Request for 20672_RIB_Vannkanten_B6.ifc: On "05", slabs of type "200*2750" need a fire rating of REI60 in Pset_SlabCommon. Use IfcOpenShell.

First a look at what the model holds.

```python
import ifcopenshell
import ifcopenshell.util.element

model = ifcopenshell.open("20672_RIB_Vannkanten_B6.ifc")
print(model.schema)
storey = next(s for s in model.by_type("IfcBuildingStorey") if s.Name == "05")
slabs = [e for e in ifcopenshell.util.element.get_decomposition(storey) if e.is_a("IfcSlab")]
seen = {}
for e in slabs:
    element_type = ifcopenshell.util.element.get_type(e)
    key = (element_type.Name if element_type != e and element_type else None, ifcopenshell.util.element.get_pset(e, "Pset_SlabCommon", "FireRating"))
    seen[key] = seen.get(key, 0) + 1
for (name, value), count in sorted(seen.items(), key=str):
    print(count, "x", name, "|", value)
```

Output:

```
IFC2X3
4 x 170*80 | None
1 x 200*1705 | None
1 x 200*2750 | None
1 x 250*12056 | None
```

```python
import ifcopenshell
import ifcopenshell.api.pset
import ifcopenshell.util.element

model = ifcopenshell.open("20672_RIB_Vannkanten_B6.ifc")

storey = next(s for s in model.by_type("IfcBuildingStorey") if s.Name == "05")
slabs = [e for e in ifcopenshell.util.element.get_decomposition(storey) if e.is_a("IfcSlab")]

count = 0
for e in slabs:
    element_type = ifcopenshell.util.element.get_type(e)
    if element_type in (None, e) or element_type.Name != "200*2750":
        continue
    # add_pset returns the element's existing set when there is one.
    pset = ifcopenshell.api.pset.add_pset(model, product=e, name="Pset_SlabCommon")
    ifcopenshell.api.pset.edit_pset(model, pset=pset, properties={"FireRating": "REI60"})
    count += 1

print(count, "slabs updated")

model.write("20672_RIB_Vannkanten_B6_v2.ifc")
```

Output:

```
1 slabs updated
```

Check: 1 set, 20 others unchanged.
